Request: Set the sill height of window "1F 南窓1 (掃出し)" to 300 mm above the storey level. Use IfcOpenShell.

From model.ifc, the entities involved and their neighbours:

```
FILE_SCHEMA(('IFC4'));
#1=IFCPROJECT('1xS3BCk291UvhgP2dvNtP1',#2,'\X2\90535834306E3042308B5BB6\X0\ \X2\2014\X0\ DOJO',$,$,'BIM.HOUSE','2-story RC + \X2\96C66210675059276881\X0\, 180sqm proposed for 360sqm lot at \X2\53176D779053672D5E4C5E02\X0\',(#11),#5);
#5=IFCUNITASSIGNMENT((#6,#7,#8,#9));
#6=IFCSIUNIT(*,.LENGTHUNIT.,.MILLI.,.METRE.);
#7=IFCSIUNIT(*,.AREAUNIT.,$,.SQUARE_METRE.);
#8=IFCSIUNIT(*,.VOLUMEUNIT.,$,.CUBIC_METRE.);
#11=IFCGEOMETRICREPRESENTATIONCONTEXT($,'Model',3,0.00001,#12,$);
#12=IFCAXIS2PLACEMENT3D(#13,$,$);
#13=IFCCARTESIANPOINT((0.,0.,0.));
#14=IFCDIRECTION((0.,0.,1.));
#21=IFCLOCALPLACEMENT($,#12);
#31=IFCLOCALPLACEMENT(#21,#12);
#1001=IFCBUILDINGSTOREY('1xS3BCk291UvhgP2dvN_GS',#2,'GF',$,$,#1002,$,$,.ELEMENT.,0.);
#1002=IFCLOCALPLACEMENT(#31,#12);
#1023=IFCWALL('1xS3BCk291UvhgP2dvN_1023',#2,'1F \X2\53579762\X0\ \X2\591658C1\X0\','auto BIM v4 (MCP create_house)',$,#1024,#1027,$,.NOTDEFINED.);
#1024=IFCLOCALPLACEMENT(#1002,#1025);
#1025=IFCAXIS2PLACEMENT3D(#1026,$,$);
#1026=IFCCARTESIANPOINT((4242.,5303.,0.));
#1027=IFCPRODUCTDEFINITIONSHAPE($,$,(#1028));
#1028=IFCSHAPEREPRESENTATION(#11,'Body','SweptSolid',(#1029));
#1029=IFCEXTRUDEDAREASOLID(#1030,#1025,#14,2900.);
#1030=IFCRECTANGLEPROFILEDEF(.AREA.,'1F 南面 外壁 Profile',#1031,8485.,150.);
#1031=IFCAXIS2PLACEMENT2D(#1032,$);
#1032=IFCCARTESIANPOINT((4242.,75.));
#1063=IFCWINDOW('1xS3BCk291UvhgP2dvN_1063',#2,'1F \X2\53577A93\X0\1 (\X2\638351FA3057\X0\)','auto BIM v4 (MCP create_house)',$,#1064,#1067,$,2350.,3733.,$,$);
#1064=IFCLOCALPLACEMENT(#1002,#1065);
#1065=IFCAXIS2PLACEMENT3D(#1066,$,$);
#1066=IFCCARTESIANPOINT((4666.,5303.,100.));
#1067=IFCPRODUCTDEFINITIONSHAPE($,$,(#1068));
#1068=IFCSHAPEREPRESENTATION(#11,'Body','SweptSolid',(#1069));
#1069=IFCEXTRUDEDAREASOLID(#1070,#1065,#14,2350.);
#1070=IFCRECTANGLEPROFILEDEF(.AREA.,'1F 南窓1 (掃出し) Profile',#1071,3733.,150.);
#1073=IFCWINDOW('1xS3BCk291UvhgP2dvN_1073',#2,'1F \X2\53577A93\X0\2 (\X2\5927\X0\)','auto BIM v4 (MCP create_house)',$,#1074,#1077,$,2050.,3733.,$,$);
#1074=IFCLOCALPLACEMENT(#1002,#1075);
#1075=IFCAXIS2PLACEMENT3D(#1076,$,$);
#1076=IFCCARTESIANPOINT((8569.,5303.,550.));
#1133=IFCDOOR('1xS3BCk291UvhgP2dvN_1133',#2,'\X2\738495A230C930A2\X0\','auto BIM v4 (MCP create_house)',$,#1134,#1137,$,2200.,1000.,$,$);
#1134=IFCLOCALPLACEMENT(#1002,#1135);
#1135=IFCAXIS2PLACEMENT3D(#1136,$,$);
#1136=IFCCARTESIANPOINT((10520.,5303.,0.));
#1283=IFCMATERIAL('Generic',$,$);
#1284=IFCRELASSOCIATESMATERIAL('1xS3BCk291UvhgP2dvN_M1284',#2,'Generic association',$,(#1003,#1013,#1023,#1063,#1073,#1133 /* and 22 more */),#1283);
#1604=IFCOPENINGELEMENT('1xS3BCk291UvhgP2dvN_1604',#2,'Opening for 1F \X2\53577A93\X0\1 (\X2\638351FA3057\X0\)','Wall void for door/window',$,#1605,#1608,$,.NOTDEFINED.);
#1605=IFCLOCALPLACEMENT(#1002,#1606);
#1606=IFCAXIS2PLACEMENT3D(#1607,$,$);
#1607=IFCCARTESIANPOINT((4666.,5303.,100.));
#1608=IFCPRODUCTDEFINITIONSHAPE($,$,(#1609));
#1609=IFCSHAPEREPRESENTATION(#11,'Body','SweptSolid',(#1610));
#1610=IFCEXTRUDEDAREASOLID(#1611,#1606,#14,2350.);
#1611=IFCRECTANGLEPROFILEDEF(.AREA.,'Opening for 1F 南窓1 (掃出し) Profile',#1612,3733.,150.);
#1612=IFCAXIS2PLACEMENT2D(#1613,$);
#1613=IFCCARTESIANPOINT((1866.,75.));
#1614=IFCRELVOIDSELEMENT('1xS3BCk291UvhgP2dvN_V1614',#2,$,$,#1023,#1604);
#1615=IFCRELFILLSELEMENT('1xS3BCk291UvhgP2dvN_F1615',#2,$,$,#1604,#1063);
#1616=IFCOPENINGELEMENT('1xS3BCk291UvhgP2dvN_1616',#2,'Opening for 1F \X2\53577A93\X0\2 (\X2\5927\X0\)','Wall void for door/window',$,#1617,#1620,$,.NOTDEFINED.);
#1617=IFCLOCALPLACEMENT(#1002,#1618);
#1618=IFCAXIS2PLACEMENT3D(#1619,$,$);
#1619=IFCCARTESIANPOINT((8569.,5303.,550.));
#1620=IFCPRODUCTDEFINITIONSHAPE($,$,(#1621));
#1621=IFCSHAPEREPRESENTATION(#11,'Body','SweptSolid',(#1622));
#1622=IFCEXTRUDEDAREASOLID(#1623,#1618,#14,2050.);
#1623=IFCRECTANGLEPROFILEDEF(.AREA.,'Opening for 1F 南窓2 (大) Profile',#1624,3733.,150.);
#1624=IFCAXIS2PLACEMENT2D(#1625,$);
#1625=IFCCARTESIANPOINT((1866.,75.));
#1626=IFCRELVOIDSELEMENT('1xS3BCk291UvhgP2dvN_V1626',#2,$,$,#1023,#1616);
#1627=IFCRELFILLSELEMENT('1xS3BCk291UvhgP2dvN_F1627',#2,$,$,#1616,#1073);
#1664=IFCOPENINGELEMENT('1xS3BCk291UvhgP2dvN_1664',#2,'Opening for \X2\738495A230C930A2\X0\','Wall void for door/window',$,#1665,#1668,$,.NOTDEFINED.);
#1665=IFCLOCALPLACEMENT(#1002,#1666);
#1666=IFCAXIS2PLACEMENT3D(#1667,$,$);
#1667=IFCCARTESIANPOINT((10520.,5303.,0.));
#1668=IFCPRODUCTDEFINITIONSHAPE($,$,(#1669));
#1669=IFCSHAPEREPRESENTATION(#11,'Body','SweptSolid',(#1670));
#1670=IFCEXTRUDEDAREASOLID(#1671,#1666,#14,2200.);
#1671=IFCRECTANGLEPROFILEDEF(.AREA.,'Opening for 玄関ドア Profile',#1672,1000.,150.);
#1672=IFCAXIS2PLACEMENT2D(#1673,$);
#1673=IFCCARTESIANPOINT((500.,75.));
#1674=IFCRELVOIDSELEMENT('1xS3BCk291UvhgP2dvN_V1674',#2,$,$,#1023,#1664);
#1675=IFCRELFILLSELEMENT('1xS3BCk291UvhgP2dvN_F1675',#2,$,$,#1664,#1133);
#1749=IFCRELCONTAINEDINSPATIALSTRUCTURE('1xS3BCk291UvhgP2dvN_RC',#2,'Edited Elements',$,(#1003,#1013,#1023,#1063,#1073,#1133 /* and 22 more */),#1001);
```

```python
import numpy as np
import ifcopenshell
import ifcopenshell.api.geometry
import ifcopenshell.geom
import ifcopenshell.util.element
import ifcopenshell.util.placement
import ifcopenshell.util.shape
import ifcopenshell.util.unit

model = ifcopenshell.open("model.ifc")
unit_scale = ifcopenshell.util.unit.calculate_unit_scale(model)

window = model.by_guid("1xS3BCk291UvhgP2dvN_1063")
opening = window.FillsVoids[0].RelatingOpeningElement
storey = ifcopenshell.util.element.get_container(window, ifc_class="IfcBuildingStorey")
level = ifcopenshell.util.placement.get_local_placement(storey.ObjectPlacement)[2, 3]

# The opening's origin need not be at the sill, so measure its lowest point.
shape = ifcopenshell.geom.create_shape(ifcopenshell.geom.settings(), opening)
bottom = ifcopenshell.util.shape.get_shape_bottom_elevation(shape, shape.geometry) / unit_scale
dz = level + 300.0 - bottom

shift = np.array([0.0, 0.0, dz])
# The window is not placed relative to its opening, so move both.
for product in (opening, window):
    matrix = ifcopenshell.util.placement.get_local_placement(product.ObjectPlacement)
    matrix[:3, 3] += shift
    ifcopenshell.api.geometry.edit_object_placement(model, product=product, matrix=matrix, is_si=False)

print(f"moved by {dz * unit_scale:+.3f} m")

model.write("model-out.ifc")
```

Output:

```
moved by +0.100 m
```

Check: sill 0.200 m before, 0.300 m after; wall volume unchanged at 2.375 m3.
